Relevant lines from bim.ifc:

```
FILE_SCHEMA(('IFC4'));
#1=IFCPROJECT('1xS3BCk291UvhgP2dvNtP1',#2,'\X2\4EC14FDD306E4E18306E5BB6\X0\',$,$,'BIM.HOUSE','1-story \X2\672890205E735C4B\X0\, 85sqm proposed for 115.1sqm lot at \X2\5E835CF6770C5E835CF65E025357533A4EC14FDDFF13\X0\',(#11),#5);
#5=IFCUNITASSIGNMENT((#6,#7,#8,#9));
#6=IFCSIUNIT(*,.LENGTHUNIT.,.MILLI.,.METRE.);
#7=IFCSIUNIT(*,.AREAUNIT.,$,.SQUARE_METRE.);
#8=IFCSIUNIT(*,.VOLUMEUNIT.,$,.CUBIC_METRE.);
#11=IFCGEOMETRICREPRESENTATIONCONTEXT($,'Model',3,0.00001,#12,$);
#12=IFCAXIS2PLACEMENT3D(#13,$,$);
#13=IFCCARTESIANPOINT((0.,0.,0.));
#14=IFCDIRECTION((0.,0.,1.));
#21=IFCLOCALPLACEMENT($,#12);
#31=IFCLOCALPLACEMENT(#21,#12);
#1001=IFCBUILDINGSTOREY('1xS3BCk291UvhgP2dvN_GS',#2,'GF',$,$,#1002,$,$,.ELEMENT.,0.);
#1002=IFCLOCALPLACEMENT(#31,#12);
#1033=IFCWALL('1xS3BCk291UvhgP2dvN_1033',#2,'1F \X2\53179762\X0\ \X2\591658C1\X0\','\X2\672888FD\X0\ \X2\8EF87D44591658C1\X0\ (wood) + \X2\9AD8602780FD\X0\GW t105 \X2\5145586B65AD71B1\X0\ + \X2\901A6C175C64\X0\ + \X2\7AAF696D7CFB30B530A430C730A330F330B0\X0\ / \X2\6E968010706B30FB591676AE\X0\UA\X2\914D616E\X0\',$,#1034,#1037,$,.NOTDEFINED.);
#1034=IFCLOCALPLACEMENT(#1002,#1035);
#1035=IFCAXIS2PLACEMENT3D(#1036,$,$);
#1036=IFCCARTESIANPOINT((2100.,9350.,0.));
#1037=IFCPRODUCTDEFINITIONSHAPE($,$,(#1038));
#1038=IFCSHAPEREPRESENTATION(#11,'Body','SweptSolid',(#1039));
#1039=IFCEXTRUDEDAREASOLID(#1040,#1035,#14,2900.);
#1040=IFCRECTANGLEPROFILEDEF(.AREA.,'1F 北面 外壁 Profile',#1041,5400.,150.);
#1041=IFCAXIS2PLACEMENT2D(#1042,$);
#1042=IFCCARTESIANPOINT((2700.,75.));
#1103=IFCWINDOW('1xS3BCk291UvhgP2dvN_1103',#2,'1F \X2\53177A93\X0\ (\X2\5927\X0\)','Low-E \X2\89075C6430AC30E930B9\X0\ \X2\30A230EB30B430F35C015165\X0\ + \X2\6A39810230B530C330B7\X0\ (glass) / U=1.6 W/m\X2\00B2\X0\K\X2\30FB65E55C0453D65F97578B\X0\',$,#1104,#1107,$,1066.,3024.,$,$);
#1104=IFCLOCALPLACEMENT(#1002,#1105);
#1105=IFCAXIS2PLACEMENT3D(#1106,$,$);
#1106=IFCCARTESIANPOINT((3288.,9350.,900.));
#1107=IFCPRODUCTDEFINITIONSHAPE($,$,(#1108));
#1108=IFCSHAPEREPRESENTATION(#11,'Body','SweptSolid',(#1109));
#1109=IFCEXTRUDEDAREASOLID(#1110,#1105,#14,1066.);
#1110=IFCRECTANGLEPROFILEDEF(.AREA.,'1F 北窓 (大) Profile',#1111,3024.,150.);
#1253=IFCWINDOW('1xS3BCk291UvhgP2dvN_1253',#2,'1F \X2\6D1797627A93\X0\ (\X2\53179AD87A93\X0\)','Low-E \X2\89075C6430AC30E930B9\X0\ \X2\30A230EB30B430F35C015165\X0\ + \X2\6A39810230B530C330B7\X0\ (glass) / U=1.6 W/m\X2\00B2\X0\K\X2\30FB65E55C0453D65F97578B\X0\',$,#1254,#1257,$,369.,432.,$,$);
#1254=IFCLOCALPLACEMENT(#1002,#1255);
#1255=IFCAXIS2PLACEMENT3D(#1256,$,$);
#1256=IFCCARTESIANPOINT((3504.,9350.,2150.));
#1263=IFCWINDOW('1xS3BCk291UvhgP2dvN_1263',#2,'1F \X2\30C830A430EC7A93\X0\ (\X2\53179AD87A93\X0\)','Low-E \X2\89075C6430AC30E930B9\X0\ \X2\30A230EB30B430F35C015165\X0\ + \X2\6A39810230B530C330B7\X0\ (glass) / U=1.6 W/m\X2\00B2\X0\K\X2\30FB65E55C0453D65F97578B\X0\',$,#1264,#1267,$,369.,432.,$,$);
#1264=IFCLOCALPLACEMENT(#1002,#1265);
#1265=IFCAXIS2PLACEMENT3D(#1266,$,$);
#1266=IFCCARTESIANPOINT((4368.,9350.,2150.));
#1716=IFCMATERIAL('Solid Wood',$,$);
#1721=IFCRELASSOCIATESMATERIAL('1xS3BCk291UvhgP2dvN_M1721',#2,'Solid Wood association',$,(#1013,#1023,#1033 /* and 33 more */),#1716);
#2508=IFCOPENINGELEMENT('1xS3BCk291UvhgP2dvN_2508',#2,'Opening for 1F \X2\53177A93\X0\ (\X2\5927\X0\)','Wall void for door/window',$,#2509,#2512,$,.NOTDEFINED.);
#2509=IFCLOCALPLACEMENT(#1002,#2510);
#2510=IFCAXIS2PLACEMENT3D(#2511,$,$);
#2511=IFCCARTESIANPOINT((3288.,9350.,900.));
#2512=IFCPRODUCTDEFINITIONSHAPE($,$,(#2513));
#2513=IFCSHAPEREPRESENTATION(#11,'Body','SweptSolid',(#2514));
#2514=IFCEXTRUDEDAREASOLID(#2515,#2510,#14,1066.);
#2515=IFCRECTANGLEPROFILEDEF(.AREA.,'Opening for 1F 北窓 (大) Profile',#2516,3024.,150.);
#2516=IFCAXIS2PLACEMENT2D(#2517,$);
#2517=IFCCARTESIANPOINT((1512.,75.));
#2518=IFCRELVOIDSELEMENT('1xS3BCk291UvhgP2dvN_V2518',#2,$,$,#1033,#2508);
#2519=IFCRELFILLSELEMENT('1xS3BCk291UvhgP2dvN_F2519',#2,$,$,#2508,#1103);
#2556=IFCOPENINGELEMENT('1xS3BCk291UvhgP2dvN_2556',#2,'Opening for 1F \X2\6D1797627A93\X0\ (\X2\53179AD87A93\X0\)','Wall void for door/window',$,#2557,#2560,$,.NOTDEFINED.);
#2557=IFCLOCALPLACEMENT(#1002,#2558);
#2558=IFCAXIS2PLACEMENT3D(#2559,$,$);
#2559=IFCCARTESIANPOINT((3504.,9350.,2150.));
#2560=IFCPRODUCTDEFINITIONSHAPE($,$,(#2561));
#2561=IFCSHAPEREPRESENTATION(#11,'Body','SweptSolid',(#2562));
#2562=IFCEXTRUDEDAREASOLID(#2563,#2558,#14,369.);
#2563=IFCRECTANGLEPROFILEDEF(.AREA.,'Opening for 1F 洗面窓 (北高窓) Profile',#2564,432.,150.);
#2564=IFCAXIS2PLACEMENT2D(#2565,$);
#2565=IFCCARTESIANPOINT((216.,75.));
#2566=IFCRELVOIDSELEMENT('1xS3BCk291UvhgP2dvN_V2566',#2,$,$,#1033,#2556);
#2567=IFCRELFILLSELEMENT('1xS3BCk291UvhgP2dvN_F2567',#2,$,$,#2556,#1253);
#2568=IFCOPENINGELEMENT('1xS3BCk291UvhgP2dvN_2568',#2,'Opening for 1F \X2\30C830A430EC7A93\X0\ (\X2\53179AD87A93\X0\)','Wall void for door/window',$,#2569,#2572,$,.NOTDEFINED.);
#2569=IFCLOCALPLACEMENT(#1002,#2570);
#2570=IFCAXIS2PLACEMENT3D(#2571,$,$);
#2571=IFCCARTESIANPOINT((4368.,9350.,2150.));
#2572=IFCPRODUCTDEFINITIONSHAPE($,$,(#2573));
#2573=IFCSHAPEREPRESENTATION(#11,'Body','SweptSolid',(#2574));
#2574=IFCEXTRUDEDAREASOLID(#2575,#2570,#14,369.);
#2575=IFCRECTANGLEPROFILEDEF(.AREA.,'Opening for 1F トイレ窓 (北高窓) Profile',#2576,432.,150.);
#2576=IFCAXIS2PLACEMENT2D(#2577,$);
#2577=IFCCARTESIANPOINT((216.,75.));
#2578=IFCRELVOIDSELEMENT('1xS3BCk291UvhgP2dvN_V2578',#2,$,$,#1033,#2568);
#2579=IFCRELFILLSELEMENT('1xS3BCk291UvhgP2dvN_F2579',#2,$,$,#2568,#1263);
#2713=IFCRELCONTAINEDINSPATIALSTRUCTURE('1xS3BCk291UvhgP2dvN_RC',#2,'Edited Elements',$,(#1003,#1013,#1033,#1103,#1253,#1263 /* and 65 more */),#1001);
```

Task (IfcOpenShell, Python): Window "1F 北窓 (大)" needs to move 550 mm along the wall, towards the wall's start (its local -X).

```python
import ifcopenshell
import ifcopenshell.api.geometry
import ifcopenshell.util.placement
import ifcopenshell.util.unit

model = ifcopenshell.open("bim.ifc")
unit_scale = ifcopenshell.util.unit.calculate_unit_scale(model)

window = model.by_guid("1xS3BCk291UvhgP2dvN_1103")
opening = window.FillsVoids[0].RelatingOpeningElement
wall = opening.VoidsElements[0].RelatingBuildingElement

wall_matrix = ifcopenshell.util.placement.get_local_placement(wall.ObjectPlacement)
shift = wall_matrix[:3, 0] * -0.55 / unit_scale
before = ifcopenshell.util.placement.get_local_placement(window.ObjectPlacement)[:3, 3].copy()

# The window is not placed relative to its opening, so move both.
for product in (opening, window):
    matrix = ifcopenshell.util.placement.get_local_placement(product.ObjectPlacement)
    matrix[:3, 3] += shift
    ifcopenshell.api.geometry.edit_object_placement(model, product=product, matrix=matrix, is_si=False)

after = ifcopenshell.util.placement.get_local_placement(window.ObjectPlacement)[:3, 3]
print("window moved by", (after - before).round(3) + 0.0)

model.write("bim_updated.ifc")
```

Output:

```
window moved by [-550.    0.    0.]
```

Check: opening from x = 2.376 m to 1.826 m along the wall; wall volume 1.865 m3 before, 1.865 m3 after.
